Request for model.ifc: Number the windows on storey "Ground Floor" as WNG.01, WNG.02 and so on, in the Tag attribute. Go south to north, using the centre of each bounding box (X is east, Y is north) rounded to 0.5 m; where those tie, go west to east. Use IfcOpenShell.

First a look at what the model holds.

```python
import ifcopenshell
import ifcopenshell.util.element
import ifcopenshell.util.placement

model = ifcopenshell.open("model.ifc")
print(model.schema)
storey = next(s for s in model.by_type("IfcBuildingStorey") if s.Name == "Ground Floor")
windows = [e for e in ifcopenshell.util.element.get_decomposition(storey) if e.is_a("IfcWindow")]
for e in sorted(windows, key=lambda e: e.id()):
    origin = ifcopenshell.util.placement.get_local_placement(e.ObjectPlacement)[:3, 3]
    print(e.id(), e.Tag, e.Name, origin.round(2) + 0.0, sep=" | ")
```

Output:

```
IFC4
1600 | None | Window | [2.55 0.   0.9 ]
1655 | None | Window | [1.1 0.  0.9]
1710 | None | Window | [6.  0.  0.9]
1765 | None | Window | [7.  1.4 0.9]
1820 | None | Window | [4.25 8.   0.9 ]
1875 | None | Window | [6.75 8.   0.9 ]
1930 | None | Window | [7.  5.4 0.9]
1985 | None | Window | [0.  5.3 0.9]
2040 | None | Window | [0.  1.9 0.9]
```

```python
import ifcopenshell
import ifcopenshell.geom
import ifcopenshell.util.element
import ifcopenshell.util.shape

model = ifcopenshell.open("model.ifc")
settings = ifcopenshell.geom.settings()
settings.set("use-world-coords", True)


def centre(element):
    shape = ifcopenshell.geom.create_shape(settings, element)
    return ifcopenshell.util.shape.get_bbox_centroid(shape.geometry)


storey = next(s for s in model.by_type("IfcBuildingStorey") if s.Name == "Ground Floor")
windows = [e for e in ifcopenshell.util.element.get_decomposition(storey) if e.is_a("IfcWindow")]

# Insertion points can sit at a corner or the storey origin, so sort by the geometry (in metres).
centres = {e: centre(e) for e in windows}
windows.sort(key=lambda e: (round(centres[e][1] / 0.5), centres[e][0]))

for i, e in enumerate(windows, start=1):
    number = f"WNG.{i:02d}"
    e.Tag = number
    print(e.id(), number)

model.write("model_v2.ifc")
```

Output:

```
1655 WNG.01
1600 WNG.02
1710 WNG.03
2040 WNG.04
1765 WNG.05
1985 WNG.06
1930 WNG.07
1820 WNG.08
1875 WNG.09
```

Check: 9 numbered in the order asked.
